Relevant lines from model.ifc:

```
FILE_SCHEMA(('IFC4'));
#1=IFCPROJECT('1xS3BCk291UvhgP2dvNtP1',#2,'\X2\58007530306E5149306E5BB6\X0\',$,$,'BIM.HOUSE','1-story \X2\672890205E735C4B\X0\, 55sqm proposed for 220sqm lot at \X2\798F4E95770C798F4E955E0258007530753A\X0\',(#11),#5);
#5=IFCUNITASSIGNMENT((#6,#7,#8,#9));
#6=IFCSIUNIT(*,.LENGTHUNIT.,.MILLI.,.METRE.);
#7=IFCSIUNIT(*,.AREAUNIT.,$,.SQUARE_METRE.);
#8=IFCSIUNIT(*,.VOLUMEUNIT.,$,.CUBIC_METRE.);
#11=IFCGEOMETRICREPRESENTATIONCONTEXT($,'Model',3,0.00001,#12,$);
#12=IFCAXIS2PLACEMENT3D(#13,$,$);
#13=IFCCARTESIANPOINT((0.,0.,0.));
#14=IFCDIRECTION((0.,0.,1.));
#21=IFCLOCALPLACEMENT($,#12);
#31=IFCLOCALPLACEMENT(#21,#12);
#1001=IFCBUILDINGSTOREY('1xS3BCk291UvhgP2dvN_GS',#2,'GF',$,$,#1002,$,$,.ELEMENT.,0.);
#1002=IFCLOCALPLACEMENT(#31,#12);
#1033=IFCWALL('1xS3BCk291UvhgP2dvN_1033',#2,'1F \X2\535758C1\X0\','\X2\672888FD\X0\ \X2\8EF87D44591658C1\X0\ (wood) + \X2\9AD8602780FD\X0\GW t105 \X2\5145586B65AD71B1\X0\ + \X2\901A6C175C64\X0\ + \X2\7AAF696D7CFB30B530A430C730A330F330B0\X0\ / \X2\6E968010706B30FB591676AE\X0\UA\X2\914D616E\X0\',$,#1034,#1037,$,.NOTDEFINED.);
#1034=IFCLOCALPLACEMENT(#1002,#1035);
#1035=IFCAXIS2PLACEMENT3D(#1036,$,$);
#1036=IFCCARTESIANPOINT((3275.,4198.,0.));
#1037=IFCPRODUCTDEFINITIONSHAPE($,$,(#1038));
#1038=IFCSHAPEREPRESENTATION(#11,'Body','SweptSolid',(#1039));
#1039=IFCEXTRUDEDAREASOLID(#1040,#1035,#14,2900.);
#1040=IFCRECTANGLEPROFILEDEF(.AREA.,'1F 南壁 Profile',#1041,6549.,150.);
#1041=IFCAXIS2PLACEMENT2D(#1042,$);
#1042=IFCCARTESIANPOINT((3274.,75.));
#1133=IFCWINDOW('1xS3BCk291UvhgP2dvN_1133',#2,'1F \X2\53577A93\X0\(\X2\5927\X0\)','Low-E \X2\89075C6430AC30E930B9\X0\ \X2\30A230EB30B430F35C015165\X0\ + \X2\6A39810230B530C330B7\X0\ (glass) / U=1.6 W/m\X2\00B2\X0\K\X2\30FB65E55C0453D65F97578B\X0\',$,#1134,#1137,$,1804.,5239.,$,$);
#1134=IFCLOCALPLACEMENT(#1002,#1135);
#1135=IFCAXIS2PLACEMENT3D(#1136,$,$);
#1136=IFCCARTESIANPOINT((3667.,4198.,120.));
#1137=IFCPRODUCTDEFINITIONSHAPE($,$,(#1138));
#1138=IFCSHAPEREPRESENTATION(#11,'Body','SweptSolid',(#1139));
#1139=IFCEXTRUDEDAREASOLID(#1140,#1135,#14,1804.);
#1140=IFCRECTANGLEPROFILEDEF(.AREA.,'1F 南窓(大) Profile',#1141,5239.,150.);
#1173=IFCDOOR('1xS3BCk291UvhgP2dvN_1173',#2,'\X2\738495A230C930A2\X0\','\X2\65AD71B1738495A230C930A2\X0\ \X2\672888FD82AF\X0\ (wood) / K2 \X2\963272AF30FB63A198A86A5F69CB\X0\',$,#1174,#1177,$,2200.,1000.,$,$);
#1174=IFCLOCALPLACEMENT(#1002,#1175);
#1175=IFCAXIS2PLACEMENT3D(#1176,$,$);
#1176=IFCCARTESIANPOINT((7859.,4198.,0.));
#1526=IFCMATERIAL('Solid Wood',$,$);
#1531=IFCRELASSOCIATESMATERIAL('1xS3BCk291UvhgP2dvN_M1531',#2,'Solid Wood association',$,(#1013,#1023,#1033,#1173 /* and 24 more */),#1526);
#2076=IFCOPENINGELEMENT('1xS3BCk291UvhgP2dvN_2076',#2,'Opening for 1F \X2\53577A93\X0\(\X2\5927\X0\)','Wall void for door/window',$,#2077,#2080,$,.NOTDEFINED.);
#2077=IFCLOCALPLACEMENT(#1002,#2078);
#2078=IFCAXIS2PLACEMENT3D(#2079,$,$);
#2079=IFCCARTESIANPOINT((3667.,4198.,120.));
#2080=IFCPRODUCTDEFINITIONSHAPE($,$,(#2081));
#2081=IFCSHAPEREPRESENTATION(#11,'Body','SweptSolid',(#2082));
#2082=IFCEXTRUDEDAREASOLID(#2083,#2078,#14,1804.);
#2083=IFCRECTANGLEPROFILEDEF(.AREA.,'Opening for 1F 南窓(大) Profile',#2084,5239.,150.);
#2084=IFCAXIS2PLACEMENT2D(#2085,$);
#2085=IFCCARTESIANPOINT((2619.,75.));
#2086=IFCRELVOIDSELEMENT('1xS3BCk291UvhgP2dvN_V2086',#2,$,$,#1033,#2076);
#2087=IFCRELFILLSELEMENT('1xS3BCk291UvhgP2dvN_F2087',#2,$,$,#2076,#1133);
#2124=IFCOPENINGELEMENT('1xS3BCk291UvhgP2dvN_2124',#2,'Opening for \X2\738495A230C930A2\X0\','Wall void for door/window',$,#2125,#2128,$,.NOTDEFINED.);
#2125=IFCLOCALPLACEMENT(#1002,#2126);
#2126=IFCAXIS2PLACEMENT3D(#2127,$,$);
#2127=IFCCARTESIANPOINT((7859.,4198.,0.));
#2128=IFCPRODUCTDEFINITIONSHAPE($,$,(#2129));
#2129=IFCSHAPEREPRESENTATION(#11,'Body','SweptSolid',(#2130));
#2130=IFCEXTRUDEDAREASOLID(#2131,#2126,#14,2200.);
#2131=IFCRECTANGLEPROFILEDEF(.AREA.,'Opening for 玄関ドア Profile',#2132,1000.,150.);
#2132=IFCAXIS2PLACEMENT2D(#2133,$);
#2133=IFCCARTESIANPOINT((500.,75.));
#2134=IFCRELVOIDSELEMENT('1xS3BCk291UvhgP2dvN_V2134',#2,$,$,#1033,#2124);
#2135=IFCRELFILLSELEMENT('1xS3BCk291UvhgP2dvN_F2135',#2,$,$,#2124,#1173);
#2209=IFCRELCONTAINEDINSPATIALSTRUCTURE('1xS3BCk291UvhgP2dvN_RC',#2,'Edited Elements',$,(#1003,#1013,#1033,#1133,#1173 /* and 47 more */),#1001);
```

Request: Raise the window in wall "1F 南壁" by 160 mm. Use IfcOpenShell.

```python
import numpy as np
import ifcopenshell
import ifcopenshell.api.geometry
import ifcopenshell.util.placement
import ifcopenshell.util.unit

model = ifcopenshell.open("model.ifc")
unit_scale = ifcopenshell.util.unit.calculate_unit_scale(model)

window = model.by_id(1133)
opening = window.FillsVoids[0].RelatingOpeningElement
dz = 0.16 / unit_scale

shift = np.array([0.0, 0.0, dz])
# The window is not placed relative to its opening, so move both.
for product in (opening, window):
    matrix = ifcopenshell.util.placement.get_local_placement(product.ObjectPlacement)
    matrix[:3, 3] += shift
    ifcopenshell.api.geometry.edit_object_placement(model, product=product, matrix=matrix, is_si=False)

print(f"moved by {dz * unit_scale:+.3f} m")

model.write("model_v2.ifc")
```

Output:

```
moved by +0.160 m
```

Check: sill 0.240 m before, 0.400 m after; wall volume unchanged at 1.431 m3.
